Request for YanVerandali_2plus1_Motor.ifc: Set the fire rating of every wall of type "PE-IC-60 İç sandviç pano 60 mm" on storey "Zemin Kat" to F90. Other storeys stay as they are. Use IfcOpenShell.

First a look at what the model holds.

```python
import ifcopenshell
import ifcopenshell.util.element

model = ifcopenshell.open("YanVerandali_2plus1_Motor.ifc")
print(model.schema)
storey = next(s for s in model.by_type("IfcBuildingStorey") if s.Name == "Zemin Kat")
walls = [e for e in ifcopenshell.util.element.get_decomposition(storey) if e.is_a("IfcWall")]
seen = {}
for e in walls:
    element_type = ifcopenshell.util.element.get_type(e)
    key = (element_type.Name if element_type != e and element_type else None, ifcopenshell.util.element.get_pset(e, "Pset_WallCommon", "FireRating"))
    seen[key] = seen.get(key, 0) + 1
for (name, value), count in sorted(seen.items(), key=str):
    print(count, "x", name, "|", value)
```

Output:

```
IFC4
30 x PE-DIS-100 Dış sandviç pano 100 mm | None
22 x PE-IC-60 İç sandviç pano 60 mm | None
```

```python
import ifcopenshell
import ifcopenshell.api.pset
import ifcopenshell.util.element

model = ifcopenshell.open("YanVerandali_2plus1_Motor.ifc")

storey = next(s for s in model.by_type("IfcBuildingStorey") if s.Name == "Zemin Kat")
walls = [e for e in ifcopenshell.util.element.get_decomposition(storey) if e.is_a("IfcWall")]

count = 0
for e in walls:
    element_type = ifcopenshell.util.element.get_type(e)
    if element_type in (None, e) or element_type.Name != "PE-IC-60 İç sandviç pano 60 mm":
        continue
    # add_pset returns the element's existing set when there is one.
    pset = ifcopenshell.api.pset.add_pset(model, product=e, name="Pset_WallCommon")
    ifcopenshell.api.pset.edit_pset(model, pset=pset, properties={"FireRating": "F90"})
    count += 1

print(count, "walls updated")

model.write("YanVerandali_2plus1_Motor-out.ifc")
```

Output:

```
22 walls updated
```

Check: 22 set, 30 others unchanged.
